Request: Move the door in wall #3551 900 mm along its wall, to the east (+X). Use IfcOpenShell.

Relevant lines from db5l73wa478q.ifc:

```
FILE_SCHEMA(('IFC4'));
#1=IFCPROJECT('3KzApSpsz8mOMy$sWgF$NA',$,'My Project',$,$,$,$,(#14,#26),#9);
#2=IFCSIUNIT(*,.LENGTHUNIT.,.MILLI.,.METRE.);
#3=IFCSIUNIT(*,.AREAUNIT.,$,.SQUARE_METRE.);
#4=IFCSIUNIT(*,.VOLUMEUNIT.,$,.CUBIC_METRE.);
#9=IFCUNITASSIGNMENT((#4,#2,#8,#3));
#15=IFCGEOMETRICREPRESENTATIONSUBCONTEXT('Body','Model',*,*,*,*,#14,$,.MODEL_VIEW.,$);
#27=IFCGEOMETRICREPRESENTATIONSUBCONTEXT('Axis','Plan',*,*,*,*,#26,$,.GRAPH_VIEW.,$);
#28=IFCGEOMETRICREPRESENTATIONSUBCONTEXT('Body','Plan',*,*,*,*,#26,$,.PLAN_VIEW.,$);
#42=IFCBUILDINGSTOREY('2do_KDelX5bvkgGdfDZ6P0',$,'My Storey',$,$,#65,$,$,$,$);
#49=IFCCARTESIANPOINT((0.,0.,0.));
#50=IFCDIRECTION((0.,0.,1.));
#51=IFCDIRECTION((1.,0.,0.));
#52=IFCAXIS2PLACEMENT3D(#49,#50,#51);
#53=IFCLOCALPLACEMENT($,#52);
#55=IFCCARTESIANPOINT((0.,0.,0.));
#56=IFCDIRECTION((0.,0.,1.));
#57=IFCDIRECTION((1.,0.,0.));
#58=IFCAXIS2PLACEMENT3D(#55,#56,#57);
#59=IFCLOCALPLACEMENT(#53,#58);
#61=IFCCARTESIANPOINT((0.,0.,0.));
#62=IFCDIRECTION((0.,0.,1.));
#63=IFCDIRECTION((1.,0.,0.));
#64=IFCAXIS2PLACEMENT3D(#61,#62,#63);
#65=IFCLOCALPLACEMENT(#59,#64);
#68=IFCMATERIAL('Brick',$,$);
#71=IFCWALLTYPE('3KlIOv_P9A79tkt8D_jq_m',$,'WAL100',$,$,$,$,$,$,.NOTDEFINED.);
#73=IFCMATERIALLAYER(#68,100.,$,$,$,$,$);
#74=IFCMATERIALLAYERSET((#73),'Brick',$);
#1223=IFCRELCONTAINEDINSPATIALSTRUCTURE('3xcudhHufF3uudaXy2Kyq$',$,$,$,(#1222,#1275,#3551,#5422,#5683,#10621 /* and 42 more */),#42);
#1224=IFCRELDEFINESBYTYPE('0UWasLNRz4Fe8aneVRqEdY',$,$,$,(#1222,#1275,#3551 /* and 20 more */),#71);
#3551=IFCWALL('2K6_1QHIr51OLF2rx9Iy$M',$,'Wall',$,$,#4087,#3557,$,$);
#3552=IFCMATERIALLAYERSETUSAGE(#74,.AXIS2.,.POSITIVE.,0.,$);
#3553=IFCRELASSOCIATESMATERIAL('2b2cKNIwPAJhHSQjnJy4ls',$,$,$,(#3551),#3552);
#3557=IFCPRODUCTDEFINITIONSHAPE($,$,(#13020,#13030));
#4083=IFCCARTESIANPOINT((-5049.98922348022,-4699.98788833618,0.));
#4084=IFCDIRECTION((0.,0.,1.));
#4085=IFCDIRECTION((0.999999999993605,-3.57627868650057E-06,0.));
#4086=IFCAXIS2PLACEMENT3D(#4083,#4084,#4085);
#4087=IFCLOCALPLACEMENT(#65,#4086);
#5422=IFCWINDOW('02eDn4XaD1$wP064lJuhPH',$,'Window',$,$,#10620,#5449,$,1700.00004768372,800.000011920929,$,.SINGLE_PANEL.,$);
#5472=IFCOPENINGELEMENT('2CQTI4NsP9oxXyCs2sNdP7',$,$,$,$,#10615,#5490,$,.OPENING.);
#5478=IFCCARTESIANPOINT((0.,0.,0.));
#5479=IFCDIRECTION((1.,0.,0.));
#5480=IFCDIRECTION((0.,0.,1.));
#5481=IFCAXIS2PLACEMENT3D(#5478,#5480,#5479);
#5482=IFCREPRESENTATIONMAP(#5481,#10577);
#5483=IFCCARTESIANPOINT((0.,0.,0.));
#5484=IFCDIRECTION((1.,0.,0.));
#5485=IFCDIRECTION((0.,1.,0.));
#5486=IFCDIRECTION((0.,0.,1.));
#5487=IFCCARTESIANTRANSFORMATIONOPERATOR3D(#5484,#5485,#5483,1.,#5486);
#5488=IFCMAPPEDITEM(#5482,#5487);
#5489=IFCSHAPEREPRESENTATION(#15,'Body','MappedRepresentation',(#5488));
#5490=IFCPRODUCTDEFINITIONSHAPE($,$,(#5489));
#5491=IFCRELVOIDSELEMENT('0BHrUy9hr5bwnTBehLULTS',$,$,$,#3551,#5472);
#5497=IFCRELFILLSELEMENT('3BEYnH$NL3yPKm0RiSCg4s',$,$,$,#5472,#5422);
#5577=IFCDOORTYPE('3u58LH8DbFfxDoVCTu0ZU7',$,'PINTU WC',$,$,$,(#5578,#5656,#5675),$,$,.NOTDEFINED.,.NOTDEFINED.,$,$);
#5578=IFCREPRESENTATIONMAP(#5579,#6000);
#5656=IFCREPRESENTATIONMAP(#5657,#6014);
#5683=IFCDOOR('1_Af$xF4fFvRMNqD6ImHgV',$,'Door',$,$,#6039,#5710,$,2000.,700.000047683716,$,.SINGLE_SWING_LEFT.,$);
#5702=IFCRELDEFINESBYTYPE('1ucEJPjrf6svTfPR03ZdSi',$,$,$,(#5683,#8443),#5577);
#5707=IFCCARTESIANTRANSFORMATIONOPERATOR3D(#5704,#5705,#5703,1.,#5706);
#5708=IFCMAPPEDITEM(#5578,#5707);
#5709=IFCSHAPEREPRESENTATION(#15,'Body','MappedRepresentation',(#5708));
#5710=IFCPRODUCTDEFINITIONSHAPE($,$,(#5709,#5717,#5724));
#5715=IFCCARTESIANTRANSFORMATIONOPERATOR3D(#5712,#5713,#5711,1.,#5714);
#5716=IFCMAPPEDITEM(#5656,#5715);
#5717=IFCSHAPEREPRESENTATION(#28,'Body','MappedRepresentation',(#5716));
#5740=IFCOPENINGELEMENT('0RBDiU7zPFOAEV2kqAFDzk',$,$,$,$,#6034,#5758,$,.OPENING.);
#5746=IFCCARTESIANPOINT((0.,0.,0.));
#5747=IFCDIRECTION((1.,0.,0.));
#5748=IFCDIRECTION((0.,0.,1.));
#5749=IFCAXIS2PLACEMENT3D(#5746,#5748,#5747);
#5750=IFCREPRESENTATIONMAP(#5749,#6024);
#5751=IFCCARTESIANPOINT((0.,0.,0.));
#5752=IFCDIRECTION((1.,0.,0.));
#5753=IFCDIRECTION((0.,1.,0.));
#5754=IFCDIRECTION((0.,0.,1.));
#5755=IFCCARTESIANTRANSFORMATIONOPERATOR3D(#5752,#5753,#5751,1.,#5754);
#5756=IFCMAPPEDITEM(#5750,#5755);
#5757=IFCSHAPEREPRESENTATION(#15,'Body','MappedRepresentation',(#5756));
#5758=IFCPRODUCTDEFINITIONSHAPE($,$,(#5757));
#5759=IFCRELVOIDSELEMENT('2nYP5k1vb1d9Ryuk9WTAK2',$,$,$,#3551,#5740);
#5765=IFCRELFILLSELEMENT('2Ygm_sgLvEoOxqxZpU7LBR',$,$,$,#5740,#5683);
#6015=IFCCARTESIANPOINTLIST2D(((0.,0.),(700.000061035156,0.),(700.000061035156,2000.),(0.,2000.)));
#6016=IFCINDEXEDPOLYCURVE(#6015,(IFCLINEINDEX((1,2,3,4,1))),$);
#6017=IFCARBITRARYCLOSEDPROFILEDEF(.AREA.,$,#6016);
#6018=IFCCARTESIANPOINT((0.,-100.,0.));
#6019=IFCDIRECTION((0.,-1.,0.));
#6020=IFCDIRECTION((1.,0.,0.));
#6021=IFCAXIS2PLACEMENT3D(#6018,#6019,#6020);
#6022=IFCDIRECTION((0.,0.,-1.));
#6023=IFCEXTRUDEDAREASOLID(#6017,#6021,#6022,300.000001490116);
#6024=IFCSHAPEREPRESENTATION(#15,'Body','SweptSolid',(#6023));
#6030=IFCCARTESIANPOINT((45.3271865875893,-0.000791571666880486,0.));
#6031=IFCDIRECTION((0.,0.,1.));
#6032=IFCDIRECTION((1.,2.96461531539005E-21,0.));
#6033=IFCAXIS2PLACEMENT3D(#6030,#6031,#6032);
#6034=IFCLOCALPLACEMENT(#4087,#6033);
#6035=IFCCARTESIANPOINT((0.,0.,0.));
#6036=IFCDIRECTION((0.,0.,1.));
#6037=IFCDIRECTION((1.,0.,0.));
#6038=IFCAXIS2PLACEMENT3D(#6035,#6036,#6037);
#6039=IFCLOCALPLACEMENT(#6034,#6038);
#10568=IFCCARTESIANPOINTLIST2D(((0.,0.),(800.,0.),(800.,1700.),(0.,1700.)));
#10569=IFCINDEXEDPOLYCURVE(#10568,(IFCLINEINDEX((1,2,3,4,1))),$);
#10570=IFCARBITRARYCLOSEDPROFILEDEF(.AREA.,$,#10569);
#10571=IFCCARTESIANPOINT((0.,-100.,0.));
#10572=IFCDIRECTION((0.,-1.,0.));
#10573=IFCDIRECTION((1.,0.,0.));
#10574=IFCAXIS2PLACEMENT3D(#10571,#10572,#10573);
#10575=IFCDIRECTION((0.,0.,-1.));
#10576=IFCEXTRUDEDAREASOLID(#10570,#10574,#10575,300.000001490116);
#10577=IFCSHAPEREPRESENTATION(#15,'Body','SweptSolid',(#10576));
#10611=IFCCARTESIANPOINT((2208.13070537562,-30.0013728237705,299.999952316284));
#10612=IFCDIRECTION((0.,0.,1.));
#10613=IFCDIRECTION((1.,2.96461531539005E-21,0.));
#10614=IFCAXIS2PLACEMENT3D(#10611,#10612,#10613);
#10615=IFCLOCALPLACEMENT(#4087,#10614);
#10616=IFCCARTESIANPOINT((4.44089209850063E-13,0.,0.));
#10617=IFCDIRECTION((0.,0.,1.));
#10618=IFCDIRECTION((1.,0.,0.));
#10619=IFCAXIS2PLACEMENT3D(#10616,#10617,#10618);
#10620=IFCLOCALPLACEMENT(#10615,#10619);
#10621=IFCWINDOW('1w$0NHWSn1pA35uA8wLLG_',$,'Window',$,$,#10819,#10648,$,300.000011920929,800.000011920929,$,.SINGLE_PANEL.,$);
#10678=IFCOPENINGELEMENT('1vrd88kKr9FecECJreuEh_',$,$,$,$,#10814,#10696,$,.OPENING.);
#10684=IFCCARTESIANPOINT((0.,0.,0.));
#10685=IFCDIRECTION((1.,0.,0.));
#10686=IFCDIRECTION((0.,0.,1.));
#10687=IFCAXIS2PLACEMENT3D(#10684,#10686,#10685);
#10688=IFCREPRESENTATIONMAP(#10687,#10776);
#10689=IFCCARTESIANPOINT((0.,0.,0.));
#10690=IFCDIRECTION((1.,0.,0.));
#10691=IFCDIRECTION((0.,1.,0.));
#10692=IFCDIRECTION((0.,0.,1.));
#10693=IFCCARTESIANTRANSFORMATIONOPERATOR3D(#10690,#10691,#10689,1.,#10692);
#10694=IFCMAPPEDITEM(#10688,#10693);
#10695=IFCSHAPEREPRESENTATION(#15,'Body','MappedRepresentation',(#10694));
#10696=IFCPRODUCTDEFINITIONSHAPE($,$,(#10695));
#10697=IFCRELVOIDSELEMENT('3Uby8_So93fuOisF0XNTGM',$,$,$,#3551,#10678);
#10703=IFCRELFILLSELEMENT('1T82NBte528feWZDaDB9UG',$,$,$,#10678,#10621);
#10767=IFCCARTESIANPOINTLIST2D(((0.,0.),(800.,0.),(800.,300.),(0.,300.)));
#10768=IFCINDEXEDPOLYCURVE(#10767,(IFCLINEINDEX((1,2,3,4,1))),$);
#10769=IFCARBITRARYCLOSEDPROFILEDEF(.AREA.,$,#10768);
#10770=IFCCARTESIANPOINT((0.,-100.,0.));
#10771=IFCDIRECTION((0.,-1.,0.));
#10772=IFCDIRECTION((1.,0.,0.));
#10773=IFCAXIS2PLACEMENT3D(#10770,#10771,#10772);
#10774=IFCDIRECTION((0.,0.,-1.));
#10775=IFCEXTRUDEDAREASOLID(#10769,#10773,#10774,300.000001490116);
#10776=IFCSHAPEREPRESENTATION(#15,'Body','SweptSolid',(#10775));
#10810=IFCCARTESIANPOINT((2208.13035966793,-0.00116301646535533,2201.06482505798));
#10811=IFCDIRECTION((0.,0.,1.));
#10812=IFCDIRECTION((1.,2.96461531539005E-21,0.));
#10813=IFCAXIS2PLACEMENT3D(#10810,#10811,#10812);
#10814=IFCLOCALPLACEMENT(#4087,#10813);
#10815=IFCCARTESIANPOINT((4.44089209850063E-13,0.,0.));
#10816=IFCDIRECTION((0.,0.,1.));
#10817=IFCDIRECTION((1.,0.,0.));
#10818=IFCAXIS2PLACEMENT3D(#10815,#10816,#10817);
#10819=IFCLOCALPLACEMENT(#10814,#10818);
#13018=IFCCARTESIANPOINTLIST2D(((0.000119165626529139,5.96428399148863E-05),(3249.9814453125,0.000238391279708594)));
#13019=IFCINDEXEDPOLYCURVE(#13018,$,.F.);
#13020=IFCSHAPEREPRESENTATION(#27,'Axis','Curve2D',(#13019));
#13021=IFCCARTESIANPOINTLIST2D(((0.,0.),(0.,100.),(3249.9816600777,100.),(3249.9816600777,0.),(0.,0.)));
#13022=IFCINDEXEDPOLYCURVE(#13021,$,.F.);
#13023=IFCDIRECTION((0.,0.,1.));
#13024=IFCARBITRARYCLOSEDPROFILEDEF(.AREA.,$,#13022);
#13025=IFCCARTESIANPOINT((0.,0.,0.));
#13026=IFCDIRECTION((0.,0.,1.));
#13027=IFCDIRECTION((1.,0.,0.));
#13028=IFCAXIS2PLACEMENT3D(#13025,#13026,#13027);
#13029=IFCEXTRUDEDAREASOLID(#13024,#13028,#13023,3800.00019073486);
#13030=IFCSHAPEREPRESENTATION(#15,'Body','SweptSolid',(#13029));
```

```python
import ifcopenshell
import ifcopenshell.api.geometry
import ifcopenshell.util.placement
import ifcopenshell.util.unit

model = ifcopenshell.open("db5l73wa478q.ifc")
unit_scale = ifcopenshell.util.unit.calculate_unit_scale(model)

door = model.by_guid("1_Af$xF4fFvRMNqD6ImHgV")
opening = door.FillsVoids[0].RelatingOpeningElement
wall = opening.VoidsElements[0].RelatingBuildingElement

wall_matrix = ifcopenshell.util.placement.get_local_placement(wall.ObjectPlacement)
shift = wall_matrix[:3, 0] * 0.9 / unit_scale
before = ifcopenshell.util.placement.get_local_placement(door.ObjectPlacement)[:3, 3].copy()

# The door is placed relative to its opening, so it follows when the opening moves.
matrix = ifcopenshell.util.placement.get_local_placement(opening.ObjectPlacement)
matrix[:3, 3] += shift
ifcopenshell.api.geometry.edit_object_placement(
    model, product=opening, matrix=matrix, is_si=False, should_transform_children=True
)

after = ifcopenshell.util.placement.get_local_placement(door.ObjectPlacement)[:3, 3]
print("door moved by", (after - before).round(3) + 0.0)

model.write("db5l73wa478q_updated.ifc")
```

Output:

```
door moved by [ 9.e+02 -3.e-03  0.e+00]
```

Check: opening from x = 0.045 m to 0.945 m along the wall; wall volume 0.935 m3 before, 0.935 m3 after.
